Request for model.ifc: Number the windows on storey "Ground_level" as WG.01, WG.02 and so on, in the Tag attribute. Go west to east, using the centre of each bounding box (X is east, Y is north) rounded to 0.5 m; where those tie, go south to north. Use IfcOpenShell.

First a look at what the model holds.

```python
import ifcopenshell
import ifcopenshell.util.element
import ifcopenshell.util.placement

model = ifcopenshell.open("model.ifc")
print(model.schema)
storey = next(s for s in model.by_type("IfcBuildingStorey") if s.Name == "Ground_level")
windows = [e for e in ifcopenshell.util.element.get_decomposition(storey) if e.is_a("IfcWindow")]
for e in sorted(windows, key=lambda e: e.id()):
    origin = ifcopenshell.util.placement.get_local_placement(e.ObjectPlacement)[:3, 3]
    print(e.id(), e.Tag, e.Name, origin.round(2) + 0.0, sep=" | ")
```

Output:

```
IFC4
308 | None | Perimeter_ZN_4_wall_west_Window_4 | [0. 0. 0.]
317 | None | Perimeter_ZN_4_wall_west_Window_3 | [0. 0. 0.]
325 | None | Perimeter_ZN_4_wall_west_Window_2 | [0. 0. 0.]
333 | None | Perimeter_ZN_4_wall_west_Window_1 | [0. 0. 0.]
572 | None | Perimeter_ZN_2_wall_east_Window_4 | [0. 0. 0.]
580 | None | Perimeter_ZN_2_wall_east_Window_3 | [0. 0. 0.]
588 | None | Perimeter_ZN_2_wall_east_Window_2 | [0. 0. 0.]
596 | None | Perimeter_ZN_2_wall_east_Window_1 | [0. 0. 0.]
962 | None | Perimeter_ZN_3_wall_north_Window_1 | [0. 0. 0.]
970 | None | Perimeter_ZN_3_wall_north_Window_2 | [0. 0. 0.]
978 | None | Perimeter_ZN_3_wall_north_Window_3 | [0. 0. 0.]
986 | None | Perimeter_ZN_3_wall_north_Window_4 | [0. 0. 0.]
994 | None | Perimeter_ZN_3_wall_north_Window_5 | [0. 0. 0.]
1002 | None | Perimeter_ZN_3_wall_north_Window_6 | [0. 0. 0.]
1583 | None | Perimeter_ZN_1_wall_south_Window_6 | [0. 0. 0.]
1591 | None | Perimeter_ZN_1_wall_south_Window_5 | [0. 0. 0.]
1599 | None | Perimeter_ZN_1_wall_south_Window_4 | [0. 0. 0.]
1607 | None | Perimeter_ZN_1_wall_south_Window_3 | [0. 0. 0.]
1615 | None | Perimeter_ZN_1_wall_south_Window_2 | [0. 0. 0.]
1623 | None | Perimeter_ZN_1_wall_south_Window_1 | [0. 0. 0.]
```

```python
import ifcopenshell
import ifcopenshell.geom
import ifcopenshell.util.element
import ifcopenshell.util.shape

model = ifcopenshell.open("model.ifc")
settings = ifcopenshell.geom.settings()
settings.set("use-world-coords", True)


def centre(element):
    shape = ifcopenshell.geom.create_shape(settings, element)
    return ifcopenshell.util.shape.get_bbox_centroid(shape.geometry)


storey = next(s for s in model.by_type("IfcBuildingStorey") if s.Name == "Ground_level")
windows = [e for e in ifcopenshell.util.element.get_decomposition(storey) if e.is_a("IfcWindow")]

# Insertion points can sit at a corner or the storey origin, so sort by the geometry (in metres).
centres = {e: centre(e) for e in windows}
windows.sort(key=lambda e: (round(centres[e][0] / 0.5), centres[e][1]))

for i, e in enumerate(windows, start=1):
    number = f"WG.{i:02d}"
    e.Tag = number
    print(e.id(), number)

model.write("model_rev.ifc")
```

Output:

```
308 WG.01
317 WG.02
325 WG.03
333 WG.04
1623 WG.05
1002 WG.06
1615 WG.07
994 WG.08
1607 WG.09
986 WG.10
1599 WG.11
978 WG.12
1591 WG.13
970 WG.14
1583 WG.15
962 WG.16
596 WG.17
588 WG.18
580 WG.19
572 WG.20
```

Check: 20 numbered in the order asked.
